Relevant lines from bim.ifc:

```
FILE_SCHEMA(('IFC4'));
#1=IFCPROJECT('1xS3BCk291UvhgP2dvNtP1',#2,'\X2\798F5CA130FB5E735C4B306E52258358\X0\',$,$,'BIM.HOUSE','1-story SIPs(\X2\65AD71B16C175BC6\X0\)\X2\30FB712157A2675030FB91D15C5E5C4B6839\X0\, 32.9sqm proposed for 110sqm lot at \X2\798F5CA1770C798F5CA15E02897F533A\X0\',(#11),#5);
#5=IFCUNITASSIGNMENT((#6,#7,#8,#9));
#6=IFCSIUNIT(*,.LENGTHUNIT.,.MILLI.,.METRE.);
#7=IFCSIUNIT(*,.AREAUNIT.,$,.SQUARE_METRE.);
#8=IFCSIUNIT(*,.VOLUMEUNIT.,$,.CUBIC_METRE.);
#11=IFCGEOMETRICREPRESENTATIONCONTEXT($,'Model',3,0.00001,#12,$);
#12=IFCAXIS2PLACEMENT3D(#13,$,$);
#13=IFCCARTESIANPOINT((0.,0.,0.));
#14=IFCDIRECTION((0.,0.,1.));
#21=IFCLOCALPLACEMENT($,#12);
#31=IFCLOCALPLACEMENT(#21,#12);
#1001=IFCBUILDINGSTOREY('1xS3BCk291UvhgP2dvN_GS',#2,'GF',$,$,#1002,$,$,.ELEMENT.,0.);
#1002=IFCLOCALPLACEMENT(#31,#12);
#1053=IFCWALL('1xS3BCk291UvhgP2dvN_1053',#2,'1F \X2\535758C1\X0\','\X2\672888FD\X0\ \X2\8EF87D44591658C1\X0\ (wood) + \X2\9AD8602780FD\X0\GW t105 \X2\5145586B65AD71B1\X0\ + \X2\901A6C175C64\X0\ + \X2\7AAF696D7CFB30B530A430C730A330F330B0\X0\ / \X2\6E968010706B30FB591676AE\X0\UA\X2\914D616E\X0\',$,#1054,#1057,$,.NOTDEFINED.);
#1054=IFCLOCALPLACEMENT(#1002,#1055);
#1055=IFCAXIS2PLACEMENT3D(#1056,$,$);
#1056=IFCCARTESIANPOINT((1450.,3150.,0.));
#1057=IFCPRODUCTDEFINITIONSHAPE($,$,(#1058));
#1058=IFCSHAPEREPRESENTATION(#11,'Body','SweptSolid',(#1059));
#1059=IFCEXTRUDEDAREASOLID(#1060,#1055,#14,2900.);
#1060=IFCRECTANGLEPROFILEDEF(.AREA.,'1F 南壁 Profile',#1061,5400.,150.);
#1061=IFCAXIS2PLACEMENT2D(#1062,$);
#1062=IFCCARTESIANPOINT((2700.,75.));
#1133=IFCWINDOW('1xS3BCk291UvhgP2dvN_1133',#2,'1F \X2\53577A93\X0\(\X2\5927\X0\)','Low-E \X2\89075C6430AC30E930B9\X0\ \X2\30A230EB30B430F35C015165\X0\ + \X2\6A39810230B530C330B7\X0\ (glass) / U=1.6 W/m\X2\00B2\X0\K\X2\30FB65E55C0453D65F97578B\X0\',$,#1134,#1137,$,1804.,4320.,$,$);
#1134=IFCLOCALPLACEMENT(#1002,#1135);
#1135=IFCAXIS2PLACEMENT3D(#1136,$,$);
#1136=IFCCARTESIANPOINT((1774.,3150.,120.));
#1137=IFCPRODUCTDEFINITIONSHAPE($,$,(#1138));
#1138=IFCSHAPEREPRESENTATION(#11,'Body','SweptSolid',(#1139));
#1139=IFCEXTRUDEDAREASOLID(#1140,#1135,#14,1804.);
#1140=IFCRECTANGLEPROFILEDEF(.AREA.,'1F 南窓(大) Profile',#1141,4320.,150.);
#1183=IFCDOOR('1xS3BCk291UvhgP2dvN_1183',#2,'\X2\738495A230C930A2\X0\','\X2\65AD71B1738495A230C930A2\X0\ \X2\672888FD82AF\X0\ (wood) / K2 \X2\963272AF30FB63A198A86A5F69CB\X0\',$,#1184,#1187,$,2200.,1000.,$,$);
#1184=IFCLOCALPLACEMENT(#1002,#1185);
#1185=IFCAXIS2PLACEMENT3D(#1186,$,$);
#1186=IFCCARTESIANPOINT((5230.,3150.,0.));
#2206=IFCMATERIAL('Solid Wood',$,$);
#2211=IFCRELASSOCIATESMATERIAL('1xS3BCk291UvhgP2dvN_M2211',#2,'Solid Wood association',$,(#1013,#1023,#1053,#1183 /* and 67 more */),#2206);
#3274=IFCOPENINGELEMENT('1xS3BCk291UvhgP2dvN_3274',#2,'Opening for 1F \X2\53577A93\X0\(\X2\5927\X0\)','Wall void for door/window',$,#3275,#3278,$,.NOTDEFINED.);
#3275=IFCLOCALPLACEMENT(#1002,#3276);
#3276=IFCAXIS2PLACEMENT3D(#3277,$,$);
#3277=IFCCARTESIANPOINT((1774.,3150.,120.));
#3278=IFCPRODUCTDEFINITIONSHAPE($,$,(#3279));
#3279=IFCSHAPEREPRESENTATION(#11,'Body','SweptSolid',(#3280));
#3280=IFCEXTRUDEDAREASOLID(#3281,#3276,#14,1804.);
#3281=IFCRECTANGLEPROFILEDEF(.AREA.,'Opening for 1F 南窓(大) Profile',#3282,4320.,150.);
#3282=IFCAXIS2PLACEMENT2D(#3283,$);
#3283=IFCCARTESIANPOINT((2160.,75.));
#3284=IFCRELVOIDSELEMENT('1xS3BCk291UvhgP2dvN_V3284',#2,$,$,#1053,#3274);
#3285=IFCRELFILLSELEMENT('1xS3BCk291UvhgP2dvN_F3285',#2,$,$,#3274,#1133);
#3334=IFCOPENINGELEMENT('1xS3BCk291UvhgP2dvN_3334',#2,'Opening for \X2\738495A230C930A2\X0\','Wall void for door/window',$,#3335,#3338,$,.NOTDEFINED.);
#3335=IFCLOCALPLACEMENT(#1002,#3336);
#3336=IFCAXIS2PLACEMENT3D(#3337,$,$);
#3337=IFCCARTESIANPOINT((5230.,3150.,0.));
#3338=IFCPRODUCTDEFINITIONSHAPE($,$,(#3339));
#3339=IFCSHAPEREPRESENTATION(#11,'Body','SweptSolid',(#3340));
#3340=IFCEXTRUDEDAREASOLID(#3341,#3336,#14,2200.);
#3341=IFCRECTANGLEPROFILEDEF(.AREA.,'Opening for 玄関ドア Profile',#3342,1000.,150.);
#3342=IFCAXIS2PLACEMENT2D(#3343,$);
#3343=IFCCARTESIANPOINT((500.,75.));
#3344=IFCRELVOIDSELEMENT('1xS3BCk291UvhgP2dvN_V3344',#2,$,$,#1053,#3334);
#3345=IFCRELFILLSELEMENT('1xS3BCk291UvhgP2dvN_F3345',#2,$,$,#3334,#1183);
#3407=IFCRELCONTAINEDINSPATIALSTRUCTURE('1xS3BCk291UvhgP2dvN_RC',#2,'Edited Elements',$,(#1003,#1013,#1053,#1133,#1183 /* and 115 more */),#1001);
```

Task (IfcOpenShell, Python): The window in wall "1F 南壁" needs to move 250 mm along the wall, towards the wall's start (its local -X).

```python
import ifcopenshell
import ifcopenshell.api.geometry
import ifcopenshell.util.placement
import ifcopenshell.util.unit

model = ifcopenshell.open("bim.ifc")
unit_scale = ifcopenshell.util.unit.calculate_unit_scale(model)

window = model.by_guid("1xS3BCk291UvhgP2dvN_1133")
opening = window.FillsVoids[0].RelatingOpeningElement
wall = opening.VoidsElements[0].RelatingBuildingElement

wall_matrix = ifcopenshell.util.placement.get_local_placement(wall.ObjectPlacement)
shift = wall_matrix[:3, 0] * -0.25 / unit_scale
before = ifcopenshell.util.placement.get_local_placement(window.ObjectPlacement)[:3, 3].copy()

# The window is not placed relative to its opening, so move both.
for product in (opening, window):
    matrix = ifcopenshell.util.placement.get_local_placement(product.ObjectPlacement)
    matrix[:3, 3] += shift
    ifcopenshell.api.geometry.edit_object_placement(model, product=product, matrix=matrix, is_si=False)

after = ifcopenshell.util.placement.get_local_placement(window.ObjectPlacement)[:3, 3]
print("window moved by", (after - before).round(3) + 0.0)

model.write("bim_rev.ifc")
```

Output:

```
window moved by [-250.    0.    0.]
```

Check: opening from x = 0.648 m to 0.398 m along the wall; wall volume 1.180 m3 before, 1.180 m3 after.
